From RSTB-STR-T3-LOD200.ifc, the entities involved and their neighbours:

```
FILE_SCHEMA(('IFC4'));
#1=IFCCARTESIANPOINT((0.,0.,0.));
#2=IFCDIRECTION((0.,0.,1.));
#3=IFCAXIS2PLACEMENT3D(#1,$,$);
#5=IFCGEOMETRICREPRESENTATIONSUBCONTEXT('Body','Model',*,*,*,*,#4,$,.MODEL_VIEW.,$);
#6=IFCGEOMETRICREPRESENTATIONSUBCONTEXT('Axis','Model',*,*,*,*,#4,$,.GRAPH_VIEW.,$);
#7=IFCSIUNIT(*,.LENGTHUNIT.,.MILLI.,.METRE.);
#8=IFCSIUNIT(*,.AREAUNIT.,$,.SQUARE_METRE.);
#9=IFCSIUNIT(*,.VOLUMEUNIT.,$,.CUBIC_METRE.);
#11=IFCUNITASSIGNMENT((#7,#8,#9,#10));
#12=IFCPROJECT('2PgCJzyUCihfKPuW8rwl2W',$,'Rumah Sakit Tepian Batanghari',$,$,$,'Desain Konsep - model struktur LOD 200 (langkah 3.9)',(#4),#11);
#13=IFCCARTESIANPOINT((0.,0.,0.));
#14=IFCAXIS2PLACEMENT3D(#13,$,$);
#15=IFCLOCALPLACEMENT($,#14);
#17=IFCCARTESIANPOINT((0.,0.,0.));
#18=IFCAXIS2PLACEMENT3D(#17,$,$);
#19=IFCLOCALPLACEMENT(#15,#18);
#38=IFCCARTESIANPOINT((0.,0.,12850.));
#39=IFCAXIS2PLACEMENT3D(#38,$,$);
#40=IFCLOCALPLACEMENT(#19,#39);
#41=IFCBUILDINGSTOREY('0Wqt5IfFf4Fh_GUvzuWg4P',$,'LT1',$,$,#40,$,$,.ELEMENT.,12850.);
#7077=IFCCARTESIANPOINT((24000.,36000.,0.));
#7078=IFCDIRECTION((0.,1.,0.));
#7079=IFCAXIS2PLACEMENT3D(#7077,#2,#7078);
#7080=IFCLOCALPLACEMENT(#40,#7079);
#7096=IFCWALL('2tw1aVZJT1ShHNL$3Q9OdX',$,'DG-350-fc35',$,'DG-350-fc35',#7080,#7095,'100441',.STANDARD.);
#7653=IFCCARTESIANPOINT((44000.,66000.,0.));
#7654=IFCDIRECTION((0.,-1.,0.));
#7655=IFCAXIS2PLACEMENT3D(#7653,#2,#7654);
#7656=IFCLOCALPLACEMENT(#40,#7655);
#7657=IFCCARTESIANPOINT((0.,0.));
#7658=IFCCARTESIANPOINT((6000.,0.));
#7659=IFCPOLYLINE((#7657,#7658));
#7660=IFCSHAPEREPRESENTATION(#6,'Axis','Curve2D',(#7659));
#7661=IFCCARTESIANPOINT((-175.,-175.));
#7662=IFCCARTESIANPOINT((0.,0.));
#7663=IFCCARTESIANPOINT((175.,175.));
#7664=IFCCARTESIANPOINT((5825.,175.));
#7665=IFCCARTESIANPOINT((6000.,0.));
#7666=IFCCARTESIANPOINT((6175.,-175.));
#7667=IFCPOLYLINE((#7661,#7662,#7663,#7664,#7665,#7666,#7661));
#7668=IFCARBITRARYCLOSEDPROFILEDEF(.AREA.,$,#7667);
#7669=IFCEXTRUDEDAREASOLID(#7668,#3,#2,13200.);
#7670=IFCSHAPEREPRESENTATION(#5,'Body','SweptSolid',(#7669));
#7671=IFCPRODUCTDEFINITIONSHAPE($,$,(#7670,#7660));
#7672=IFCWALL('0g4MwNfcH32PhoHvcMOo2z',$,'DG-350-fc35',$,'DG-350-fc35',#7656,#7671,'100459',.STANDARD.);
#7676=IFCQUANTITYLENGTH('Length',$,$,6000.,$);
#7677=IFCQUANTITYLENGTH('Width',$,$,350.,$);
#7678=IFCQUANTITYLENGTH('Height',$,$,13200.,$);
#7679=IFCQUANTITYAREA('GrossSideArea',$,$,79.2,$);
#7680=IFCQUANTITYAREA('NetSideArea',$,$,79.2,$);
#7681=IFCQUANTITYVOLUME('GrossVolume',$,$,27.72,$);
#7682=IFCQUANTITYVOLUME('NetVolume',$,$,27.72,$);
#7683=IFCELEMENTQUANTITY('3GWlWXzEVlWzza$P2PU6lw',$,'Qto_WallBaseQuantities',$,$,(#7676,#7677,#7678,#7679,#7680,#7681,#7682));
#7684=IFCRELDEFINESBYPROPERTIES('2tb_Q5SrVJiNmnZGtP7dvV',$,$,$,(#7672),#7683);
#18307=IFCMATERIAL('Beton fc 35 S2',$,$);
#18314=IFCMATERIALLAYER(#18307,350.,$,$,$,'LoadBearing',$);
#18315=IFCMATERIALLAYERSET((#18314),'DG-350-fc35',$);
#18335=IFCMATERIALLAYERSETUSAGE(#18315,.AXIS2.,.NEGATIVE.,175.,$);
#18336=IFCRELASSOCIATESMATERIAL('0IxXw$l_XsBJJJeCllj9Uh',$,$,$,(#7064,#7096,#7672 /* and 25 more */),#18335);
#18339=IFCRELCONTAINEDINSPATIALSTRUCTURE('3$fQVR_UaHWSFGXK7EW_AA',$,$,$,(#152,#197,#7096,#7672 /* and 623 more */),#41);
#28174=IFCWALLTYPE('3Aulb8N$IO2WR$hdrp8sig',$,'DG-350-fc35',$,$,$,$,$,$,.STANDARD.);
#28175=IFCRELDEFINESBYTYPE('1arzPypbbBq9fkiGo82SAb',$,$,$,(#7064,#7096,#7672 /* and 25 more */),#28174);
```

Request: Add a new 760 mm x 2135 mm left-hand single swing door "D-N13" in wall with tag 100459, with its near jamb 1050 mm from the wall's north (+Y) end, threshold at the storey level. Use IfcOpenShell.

```python
import numpy as np
import ifcopenshell
import ifcopenshell.api.feature
import ifcopenshell.api.geometry
import ifcopenshell.api.pset
import ifcopenshell.api.root
import ifcopenshell.api.spatial
import ifcopenshell.geom
import ifcopenshell.util.element
import ifcopenshell.util.placement
import ifcopenshell.util.representation
import ifcopenshell.util.shape
import ifcopenshell.util.unit

model = ifcopenshell.open("RSTB-STR-T3-LOD200.ifc")
unit_scale = ifcopenshell.util.unit.calculate_unit_scale(model)
area_scale = ifcopenshell.util.unit.calculate_unit_scale(model, "AREAUNIT")
volume_scale = ifcopenshell.util.unit.calculate_unit_scale(model, "VOLUMEUNIT")
settings = ifcopenshell.geom.settings()


def volume(element):
    """Net volume in cubic metres, openings subtracted."""
    shape = ifcopenshell.geom.create_shape(settings, element)
    return ifcopenshell.util.shape.get_volume(shape.geometry)


wall = model.by_guid("0g4MwNfcH32PhoHvcMOo2z")
storey = ifcopenshell.util.element.get_container(wall, ifc_class="IfcBuildingStorey")
context = ifcopenshell.util.representation.get_context(model, "Model", "Body", "MODEL_VIEW")
before = volume(wall)

width, height, from_end, sill = 0.76, 2.135, 1.05, 0.0  # metres

# The wall runs along its own X axis, and the end named is its -X end.
wall_shape = ifcopenshell.geom.create_shape(settings, wall)
x, y, z = ifcopenshell.util.shape.get_vertices(wall_shape.geometry).T
start = x.min() + from_end
face, thickness = float(y.min()), float(y.max() - y.min())
wall_matrix = ifcopenshell.util.placement.get_local_placement(wall.ObjectPlacement)
level = ifcopenshell.util.placement.get_local_placement(storey.ObjectPlacement)[2, 3]


def in_wall(x, y):
    """Placement at x, y metres in the wall's axes, at sill height."""
    matrix = wall_matrix.copy()
    matrix[:, 3] = wall_matrix @ np.array([x / unit_scale, y / unit_scale, 0.0, 1.0])
    matrix[2, 3] = level + sill / unit_scale
    return matrix


# Opening: a box that overshoots both wall faces by 50 mm.
opening = ifcopenshell.api.root.create_entity(model, ifc_class="IfcOpeningElement", predefined_type="OPENING")
box = ifcopenshell.api.geometry.add_wall_representation(
    model, context=context, length=width, height=height, thickness=thickness + 0.1
)
ifcopenshell.api.geometry.assign_representation(model, product=opening, representation=box)
ifcopenshell.api.geometry.edit_object_placement(model, product=opening, matrix=in_wall(start, face - 0.05), is_si=False)
ifcopenshell.api.feature.add_feature(model, feature=opening, element=wall)

door = ifcopenshell.api.root.create_entity(model, ifc_class="IfcDoor", name="D-N13", predefined_type="DOOR")
door.OverallWidth, door.OverallHeight = width / unit_scale, height / unit_scale
door.OperationType = "SINGLE_SWING_LEFT"
body = ifcopenshell.api.geometry.add_door_representation(
    model,
    context=context,
    overall_width=door.OverallWidth,
    overall_height=door.OverallHeight,
    operation_type="SINGLE_SWING_LEFT",
    lining_properties={"LiningDepth": thickness / unit_scale, "ThresholdDepth": thickness / unit_scale},
)
ifcopenshell.api.geometry.assign_representation(model, product=door, representation=body)
ifcopenshell.api.spatial.assign_container(model, products=[door], relating_structure=storey)
ifcopenshell.api.feature.add_filling(model, opening=opening, element=door)

# The lining spans the wall, so the door starts at the wall face.
ifcopenshell.api.geometry.edit_object_placement(model, product=door, matrix=in_wall(start, face), is_si=False)

after = volume(wall)

# Update the wall's stored quantities.
qto = model.by_id(ifcopenshell.util.element.get_pset(wall, "Qto_WallBaseQuantities", should_inherit=False)["id"])
ifcopenshell.api.pset.edit_qto(model, qto=qto, properties={
    "NetSideArea": after / thickness / area_scale,
    "NetVolume": after / volume_scale,
})

print(f"wall volume {before:.3f} -> {after:.3f} m3")

model.write("RSTB-STR-T3-LOD200_edited.ifc")
```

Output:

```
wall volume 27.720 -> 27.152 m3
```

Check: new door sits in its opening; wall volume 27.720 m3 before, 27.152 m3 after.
